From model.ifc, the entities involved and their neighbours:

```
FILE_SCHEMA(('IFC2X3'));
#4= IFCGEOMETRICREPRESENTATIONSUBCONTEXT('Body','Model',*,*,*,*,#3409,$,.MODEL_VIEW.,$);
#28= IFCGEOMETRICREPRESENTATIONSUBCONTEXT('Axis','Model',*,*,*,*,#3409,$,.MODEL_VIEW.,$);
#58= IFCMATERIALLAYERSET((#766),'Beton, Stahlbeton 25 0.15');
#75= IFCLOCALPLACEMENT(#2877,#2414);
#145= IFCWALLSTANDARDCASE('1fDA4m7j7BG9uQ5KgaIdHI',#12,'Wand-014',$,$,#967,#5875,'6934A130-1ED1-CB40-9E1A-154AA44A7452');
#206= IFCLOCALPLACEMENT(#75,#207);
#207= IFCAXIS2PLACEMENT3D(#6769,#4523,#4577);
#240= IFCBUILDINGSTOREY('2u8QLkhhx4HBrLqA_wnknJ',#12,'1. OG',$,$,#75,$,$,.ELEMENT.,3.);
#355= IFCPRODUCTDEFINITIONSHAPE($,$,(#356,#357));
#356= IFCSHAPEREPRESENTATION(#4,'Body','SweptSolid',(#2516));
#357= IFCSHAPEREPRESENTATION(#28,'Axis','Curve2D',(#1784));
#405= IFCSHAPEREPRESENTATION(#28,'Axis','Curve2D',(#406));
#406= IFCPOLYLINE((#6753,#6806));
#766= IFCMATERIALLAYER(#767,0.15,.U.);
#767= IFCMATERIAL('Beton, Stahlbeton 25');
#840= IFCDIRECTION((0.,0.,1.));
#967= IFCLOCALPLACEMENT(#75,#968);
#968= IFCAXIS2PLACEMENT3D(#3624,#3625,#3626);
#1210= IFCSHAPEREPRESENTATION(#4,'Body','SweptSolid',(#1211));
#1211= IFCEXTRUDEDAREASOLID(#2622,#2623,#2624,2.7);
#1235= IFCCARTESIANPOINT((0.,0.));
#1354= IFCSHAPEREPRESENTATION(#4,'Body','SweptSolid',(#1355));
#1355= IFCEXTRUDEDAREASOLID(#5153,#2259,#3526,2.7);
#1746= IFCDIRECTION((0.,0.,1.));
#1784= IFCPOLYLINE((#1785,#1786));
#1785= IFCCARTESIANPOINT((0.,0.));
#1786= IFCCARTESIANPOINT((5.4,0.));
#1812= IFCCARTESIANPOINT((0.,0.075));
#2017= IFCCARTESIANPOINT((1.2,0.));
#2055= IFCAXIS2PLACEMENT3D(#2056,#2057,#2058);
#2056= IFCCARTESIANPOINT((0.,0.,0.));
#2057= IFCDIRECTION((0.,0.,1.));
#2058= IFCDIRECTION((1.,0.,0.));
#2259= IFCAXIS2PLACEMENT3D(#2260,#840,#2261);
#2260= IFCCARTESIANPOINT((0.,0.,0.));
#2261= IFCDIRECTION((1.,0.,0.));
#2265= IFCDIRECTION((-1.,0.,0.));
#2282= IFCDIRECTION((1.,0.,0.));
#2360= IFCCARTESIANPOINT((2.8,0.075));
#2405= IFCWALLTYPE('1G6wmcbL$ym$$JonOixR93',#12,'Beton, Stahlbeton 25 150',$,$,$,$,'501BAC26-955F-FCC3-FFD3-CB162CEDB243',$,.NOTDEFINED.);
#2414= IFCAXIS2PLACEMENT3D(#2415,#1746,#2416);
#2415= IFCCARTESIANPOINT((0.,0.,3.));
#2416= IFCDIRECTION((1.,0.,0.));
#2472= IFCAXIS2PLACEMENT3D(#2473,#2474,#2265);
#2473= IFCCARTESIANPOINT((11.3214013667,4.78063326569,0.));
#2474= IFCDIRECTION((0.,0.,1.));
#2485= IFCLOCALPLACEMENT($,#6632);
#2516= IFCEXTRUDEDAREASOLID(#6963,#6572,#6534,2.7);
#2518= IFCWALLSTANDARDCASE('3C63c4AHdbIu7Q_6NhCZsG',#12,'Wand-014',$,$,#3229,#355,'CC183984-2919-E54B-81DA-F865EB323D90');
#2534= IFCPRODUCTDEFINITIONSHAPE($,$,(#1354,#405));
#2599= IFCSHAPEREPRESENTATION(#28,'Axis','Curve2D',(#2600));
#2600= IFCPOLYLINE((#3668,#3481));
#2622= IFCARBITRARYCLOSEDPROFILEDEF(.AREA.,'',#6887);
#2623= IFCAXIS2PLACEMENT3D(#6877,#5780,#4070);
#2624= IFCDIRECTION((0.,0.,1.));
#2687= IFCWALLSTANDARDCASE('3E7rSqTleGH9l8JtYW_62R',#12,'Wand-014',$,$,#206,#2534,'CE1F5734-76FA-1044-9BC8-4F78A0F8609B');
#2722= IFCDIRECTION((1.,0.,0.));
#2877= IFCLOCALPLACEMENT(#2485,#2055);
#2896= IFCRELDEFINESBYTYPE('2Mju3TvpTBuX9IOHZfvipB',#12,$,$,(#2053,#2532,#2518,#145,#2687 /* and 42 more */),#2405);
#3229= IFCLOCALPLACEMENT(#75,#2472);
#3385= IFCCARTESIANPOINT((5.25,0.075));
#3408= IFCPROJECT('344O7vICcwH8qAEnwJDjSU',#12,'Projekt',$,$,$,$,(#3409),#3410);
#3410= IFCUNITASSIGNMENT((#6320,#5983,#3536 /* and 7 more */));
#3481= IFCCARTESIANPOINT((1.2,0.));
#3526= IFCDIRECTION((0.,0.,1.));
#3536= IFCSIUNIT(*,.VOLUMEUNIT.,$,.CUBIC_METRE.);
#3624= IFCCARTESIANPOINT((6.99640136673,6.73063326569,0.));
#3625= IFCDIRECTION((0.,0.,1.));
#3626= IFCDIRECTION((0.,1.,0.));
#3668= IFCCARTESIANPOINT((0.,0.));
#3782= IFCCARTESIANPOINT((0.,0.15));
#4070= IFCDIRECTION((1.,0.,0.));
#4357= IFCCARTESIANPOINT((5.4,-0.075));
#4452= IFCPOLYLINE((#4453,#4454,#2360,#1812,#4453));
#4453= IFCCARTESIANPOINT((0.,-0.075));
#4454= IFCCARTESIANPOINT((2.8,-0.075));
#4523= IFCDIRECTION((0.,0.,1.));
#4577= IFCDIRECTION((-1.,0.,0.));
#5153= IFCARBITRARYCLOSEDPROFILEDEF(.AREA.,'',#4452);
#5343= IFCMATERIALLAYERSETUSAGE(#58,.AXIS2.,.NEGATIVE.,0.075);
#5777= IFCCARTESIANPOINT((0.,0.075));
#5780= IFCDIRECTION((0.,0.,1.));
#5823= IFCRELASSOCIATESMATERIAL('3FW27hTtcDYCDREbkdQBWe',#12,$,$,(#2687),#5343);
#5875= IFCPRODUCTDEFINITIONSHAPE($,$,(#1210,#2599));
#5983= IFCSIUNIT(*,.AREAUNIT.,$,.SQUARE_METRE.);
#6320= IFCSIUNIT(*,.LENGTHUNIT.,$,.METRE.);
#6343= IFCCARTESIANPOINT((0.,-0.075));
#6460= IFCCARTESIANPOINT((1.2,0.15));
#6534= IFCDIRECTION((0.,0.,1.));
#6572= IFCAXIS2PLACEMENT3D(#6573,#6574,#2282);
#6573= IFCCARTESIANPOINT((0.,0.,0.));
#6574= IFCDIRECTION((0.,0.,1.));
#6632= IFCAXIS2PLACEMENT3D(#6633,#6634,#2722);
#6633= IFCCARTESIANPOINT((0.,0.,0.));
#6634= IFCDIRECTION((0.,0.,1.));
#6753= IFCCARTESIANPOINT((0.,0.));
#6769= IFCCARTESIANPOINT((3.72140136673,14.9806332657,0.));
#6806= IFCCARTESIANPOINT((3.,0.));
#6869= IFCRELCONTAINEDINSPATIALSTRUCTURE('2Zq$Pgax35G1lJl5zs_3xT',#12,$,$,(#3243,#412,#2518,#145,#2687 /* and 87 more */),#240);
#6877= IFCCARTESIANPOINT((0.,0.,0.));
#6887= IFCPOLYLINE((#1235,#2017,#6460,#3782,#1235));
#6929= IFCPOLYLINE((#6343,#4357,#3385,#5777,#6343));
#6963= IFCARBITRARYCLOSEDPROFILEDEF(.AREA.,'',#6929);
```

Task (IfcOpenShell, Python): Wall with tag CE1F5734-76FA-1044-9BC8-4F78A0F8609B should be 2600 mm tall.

```python
import ifcopenshell
import ifcopenshell.geom
import ifcopenshell.util.representation
import ifcopenshell.util.shape

model = ifcopenshell.open("model.ifc")
settings = ifcopenshell.geom.settings()


def volume(element):
    """Net volume in cubic metres, openings subtracted."""
    shape = ifcopenshell.geom.create_shape(settings, element)
    return ifcopenshell.util.shape.get_volume(shape.geometry)


wall = model.by_guid("3E7rSqTleGH9l8JtYW_62R")
before = volume(wall)

body = ifcopenshell.util.representation.get_representation(wall, "Model", "Body")
solid = body.Items[0]
old_height = solid.Depth
solid.Depth = 2.6
after = volume(wall)

print(f"height {old_height:g} -> {solid.Depth:g}, volume {before:.3f} -> {after:.3f} m3")

model.write("model_edited.ifc")
```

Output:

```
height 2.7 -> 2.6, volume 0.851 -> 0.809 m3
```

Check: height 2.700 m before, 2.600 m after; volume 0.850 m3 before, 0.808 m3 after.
